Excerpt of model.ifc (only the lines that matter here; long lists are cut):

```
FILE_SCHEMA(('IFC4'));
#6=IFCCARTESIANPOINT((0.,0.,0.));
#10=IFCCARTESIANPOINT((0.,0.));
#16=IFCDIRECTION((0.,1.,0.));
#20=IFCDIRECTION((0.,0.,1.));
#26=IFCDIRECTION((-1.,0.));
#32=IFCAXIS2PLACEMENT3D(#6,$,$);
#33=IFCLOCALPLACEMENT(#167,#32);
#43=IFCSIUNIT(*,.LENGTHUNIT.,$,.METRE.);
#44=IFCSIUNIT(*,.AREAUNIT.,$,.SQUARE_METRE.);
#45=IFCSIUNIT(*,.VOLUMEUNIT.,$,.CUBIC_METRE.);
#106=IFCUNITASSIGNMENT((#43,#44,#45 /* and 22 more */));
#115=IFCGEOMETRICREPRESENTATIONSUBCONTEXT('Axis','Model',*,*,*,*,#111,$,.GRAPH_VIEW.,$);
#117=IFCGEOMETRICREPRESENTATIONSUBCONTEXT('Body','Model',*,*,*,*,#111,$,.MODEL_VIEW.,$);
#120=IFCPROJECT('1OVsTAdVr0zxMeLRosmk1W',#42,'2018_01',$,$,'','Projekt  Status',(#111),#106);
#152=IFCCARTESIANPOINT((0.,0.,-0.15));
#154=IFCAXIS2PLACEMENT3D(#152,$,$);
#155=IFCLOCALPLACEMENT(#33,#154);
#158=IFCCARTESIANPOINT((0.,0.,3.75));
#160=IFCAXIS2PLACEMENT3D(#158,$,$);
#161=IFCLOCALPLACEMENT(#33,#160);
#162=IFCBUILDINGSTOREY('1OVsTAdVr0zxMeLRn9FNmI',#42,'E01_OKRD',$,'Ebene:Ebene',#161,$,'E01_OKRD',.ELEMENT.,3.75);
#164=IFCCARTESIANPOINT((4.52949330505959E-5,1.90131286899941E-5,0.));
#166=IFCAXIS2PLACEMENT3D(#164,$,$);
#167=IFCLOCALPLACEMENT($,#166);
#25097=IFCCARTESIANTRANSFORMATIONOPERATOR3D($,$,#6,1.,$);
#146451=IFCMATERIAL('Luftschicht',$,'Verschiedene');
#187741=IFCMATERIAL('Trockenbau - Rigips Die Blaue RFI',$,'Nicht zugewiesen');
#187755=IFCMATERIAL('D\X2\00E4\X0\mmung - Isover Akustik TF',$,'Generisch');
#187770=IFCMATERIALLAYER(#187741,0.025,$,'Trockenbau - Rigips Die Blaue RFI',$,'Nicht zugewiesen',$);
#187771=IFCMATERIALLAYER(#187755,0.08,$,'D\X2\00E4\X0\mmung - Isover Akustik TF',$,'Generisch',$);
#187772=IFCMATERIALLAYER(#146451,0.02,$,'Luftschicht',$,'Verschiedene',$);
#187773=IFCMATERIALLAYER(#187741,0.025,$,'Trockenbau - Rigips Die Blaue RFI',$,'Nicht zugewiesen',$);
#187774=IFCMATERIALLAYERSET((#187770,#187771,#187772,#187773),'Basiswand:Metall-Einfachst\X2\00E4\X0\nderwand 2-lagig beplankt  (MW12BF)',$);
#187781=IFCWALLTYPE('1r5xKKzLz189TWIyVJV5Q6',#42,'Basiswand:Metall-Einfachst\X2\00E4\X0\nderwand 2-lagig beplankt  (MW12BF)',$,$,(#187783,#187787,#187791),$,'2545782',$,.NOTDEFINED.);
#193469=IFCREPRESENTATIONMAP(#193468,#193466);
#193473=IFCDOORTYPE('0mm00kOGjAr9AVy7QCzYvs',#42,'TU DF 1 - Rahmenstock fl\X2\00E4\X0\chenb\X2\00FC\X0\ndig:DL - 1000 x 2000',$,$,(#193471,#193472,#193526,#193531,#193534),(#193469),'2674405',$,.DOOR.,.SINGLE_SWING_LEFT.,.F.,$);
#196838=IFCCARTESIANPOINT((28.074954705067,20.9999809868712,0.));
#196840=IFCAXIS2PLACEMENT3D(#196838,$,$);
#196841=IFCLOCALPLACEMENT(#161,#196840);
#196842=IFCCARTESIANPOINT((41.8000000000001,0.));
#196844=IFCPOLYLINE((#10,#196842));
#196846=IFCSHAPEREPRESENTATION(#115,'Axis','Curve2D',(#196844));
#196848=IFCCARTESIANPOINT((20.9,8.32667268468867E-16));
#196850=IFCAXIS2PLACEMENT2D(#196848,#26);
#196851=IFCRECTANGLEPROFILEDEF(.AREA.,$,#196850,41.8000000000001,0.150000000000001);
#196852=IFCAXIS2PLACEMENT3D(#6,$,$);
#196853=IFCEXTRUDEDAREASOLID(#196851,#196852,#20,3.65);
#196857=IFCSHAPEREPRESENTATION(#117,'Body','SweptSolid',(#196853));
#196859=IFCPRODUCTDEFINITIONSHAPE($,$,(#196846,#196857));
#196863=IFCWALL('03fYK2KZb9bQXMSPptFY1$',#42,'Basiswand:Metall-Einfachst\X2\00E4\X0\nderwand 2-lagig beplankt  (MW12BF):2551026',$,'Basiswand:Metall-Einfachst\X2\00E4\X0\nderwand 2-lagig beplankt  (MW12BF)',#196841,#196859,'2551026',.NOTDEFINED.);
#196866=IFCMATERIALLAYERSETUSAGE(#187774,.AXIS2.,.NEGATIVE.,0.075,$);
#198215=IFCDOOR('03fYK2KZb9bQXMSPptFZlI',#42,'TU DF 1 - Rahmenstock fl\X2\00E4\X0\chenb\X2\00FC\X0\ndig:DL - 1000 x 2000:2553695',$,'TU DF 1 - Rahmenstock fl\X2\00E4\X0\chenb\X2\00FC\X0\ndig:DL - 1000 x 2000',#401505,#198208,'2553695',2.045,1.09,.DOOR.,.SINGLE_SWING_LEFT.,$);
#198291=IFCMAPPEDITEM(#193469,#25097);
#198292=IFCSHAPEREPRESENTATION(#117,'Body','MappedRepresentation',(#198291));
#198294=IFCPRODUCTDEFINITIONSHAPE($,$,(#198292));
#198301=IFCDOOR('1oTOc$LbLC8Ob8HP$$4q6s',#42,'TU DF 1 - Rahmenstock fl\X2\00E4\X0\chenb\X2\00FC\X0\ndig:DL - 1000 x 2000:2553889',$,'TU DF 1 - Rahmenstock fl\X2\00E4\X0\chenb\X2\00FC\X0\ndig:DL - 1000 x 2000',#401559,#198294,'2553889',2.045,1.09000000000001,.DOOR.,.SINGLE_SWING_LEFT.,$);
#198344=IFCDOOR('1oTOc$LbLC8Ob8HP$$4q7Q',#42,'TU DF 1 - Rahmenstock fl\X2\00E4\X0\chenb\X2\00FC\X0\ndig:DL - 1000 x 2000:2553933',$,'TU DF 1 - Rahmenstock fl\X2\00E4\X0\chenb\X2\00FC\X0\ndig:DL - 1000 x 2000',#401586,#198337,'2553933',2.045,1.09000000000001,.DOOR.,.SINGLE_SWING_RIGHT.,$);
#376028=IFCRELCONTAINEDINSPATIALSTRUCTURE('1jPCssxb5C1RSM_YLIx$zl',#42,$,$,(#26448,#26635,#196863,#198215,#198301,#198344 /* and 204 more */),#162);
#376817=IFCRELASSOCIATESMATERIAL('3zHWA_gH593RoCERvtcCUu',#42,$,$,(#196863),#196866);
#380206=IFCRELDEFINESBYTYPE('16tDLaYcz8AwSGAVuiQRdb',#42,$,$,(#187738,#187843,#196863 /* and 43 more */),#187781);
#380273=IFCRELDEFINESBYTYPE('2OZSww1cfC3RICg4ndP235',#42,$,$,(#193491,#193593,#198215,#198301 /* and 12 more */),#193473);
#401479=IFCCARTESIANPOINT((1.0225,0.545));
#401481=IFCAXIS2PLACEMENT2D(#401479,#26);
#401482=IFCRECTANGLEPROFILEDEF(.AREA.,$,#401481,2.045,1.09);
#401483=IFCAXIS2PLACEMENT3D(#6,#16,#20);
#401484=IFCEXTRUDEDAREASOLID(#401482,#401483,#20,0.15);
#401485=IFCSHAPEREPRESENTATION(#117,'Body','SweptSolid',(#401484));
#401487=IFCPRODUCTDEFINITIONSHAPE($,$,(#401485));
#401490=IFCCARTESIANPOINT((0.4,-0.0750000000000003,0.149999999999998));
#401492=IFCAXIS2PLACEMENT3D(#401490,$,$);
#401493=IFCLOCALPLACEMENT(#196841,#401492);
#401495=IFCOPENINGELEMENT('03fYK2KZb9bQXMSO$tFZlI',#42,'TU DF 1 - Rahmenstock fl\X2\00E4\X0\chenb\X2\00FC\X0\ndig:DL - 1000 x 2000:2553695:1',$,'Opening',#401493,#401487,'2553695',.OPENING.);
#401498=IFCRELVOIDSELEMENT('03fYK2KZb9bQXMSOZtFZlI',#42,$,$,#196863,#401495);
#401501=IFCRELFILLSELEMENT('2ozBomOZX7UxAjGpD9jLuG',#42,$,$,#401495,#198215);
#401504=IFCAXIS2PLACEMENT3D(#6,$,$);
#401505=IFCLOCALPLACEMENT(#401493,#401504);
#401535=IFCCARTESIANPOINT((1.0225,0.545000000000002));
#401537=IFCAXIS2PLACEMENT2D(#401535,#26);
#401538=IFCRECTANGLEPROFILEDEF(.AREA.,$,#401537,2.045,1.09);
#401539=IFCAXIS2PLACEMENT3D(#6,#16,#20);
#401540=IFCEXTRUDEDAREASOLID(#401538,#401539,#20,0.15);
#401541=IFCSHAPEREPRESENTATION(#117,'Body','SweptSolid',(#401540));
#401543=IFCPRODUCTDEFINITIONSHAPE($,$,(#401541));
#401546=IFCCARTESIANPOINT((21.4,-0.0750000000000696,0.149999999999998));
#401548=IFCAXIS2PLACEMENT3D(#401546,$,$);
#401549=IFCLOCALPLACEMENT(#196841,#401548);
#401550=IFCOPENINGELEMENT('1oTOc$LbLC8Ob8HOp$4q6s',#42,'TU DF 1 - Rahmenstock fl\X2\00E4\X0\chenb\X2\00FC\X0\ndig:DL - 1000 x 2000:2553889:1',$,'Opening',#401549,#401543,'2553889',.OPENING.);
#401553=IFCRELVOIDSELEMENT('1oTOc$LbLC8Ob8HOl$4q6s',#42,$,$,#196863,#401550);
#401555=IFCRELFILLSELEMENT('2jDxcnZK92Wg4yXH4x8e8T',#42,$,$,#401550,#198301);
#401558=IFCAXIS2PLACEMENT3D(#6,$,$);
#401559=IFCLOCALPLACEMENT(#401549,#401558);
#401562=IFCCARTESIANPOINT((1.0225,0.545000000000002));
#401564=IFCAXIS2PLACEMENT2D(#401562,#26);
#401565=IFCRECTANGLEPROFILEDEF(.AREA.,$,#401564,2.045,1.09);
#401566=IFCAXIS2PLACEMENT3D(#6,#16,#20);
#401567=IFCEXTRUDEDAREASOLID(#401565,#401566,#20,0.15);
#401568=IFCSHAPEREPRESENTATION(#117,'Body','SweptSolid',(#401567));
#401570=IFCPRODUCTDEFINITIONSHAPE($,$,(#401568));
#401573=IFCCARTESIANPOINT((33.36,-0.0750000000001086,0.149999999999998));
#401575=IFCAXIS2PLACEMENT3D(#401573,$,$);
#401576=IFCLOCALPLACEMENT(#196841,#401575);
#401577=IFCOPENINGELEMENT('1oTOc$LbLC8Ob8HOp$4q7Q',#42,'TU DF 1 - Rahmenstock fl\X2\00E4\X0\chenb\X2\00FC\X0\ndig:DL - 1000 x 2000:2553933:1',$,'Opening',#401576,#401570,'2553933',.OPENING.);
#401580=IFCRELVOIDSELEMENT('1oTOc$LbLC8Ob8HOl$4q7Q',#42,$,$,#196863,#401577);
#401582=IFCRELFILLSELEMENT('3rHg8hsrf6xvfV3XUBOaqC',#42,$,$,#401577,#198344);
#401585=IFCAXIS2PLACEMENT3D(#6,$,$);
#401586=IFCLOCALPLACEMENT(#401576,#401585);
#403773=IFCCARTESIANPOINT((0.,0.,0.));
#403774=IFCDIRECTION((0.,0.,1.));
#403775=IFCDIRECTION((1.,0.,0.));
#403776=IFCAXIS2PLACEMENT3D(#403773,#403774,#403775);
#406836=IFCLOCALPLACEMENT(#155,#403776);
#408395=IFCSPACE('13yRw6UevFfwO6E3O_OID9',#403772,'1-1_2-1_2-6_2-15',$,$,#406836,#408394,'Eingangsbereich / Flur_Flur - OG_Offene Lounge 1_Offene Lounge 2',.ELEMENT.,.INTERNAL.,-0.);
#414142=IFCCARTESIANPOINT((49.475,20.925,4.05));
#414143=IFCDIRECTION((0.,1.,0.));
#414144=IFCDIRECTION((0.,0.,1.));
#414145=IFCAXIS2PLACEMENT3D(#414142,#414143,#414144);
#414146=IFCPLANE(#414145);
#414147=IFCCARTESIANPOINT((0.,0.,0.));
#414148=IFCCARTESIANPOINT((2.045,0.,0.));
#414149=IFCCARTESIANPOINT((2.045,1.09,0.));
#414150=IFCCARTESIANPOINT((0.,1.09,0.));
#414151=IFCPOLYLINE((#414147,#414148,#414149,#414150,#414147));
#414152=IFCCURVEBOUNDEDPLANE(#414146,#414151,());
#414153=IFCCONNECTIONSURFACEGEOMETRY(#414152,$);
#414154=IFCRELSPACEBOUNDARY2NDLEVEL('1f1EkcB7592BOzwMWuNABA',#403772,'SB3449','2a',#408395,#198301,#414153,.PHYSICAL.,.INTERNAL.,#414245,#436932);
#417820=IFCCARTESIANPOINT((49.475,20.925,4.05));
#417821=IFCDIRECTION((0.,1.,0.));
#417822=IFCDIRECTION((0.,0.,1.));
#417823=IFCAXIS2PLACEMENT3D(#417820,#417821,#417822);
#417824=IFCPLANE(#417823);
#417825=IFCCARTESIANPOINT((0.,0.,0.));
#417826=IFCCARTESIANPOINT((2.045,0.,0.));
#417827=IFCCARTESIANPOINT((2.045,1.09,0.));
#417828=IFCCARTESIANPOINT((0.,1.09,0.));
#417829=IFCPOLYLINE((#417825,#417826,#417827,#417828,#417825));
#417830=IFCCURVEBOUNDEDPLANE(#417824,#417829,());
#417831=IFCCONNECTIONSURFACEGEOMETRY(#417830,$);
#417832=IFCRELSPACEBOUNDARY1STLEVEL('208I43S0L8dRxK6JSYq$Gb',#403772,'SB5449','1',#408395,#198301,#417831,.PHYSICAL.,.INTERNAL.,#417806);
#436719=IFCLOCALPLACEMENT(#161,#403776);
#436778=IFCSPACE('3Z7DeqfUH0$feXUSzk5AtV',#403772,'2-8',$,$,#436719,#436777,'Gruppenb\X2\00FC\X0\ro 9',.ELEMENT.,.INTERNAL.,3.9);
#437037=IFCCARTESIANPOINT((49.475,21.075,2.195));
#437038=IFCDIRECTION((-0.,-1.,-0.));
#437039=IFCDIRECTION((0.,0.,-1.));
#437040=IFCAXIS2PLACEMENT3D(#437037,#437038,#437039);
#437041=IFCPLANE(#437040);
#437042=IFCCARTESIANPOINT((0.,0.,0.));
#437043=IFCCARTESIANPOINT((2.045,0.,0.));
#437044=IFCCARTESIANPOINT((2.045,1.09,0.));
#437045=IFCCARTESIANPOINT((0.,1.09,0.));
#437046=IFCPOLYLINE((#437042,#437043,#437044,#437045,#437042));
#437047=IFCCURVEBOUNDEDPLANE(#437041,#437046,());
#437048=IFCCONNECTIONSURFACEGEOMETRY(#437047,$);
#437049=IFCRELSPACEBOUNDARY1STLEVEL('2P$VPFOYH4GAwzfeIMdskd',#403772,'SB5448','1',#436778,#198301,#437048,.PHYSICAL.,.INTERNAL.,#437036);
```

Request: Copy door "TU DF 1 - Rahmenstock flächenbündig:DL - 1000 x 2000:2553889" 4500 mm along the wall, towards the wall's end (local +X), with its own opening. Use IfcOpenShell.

```python
import numpy as np
import ifcopenshell
import ifcopenshell.api.feature
import ifcopenshell.api.geometry
import ifcopenshell.api.root
import ifcopenshell.geom
import ifcopenshell.util.element
import ifcopenshell.util.placement
import ifcopenshell.util.shape

model = ifcopenshell.open("model.ifc")
settings = ifcopenshell.geom.settings()


def volume(element):
    """Net volume in cubic metres, openings subtracted."""
    shape = ifcopenshell.geom.create_shape(settings, element)
    return ifcopenshell.util.shape.get_volume(shape.geometry)


def reuse_history(source, copy):
    """copy_class also copies each property set's owner history, people and application; keep the originals."""
    for rel in copy.IsDefinedBy:
        if rel.is_a("IfcRelDefinesByProperties") and (history := rel.RelatingPropertyDefinition.OwnerHistory):
            rel.RelatingPropertyDefinition.OwnerHistory = source.OwnerHistory
            ifcopenshell.util.element.remove_deep2(model, history)


door = model.by_guid("1oTOc$LbLC8Ob8HP$$4q6s")
opening = door.FillsVoids[0].RelatingOpeningElement
wall = opening.VoidsElements[0].RelatingBuildingElement
before = volume(wall)
shift = ifcopenshell.util.placement.get_local_placement(wall.ObjectPlacement)[:3, 0] * 4.5

# copy_class copies the void relationship, type, container and properties, but no geometry.
new_opening = ifcopenshell.api.root.copy_class(model, product=opening)
new_opening.Representation = ifcopenshell.util.element.copy_deep(
    model, opening.Representation, exclude=["IfcGeometricRepresentationContext", "IfcRepresentationMap"]
)
new_opening.Name = "TU DF 1 - Rahmenstock flächenbündig:DL - 1000 x 2000"
new_opening.Tag = None
new_door = ifcopenshell.api.root.copy_class(model, product=door)
new_door.Representation = ifcopenshell.util.element.copy_deep(
    model, door.Representation, exclude=["IfcGeometricRepresentationContext", "IfcRepresentationMap"]
)
new_door.Name = "TU DF 1 - Rahmenstock flächenbündig:DL - 1000 x 2000"
new_door.Tag = None
reuse_history(door, new_door)
ifcopenshell.api.feature.add_filling(model, opening=new_opening, element=new_door)

for old, new in ((opening, new_opening), (door, new_door)):
    matrix = ifcopenshell.util.placement.get_local_placement(old.ObjectPlacement)
    matrix[:3, 3] += shift
    ifcopenshell.api.geometry.edit_object_placement(model, product=new, matrix=matrix, is_si=False)

# The copied space boundaries still share their surfaces with the original.
for rel in new_door.ProvidesBoundaries:
    if rel.ConnectionGeometry:
        rel.ConnectionGeometry = ifcopenshell.util.element.copy_deep(model, rel.ConnectionGeometry)

# Space boundary surfaces are stored in each space's coordinates; move them too.
for rel in new_door.ProvidesBoundaries:
    if not rel.ConnectionGeometry:
        continue
    surface = rel.ConnectionGeometry.SurfaceOnRelatingElement.BasisSurface
    space_matrix = ifcopenshell.util.placement.get_local_placement(rel.RelatingSpace.ObjectPlacement)
    point = np.array(surface.Position.Location.Coordinates) + space_matrix[:3, :3].T @ shift
    surface.Position = model.createIfcAxis2Placement3D(
        model.createIfcCartesianPoint(point.tolist()), surface.Position.Axis, surface.Position.RefDirection
    )

after = volume(wall)

print(f"wall volume {before:.3f} -> {after:.3f} m3")

model.write("model_rev.ifc")
```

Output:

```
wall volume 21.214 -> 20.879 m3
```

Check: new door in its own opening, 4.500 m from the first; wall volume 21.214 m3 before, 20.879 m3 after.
